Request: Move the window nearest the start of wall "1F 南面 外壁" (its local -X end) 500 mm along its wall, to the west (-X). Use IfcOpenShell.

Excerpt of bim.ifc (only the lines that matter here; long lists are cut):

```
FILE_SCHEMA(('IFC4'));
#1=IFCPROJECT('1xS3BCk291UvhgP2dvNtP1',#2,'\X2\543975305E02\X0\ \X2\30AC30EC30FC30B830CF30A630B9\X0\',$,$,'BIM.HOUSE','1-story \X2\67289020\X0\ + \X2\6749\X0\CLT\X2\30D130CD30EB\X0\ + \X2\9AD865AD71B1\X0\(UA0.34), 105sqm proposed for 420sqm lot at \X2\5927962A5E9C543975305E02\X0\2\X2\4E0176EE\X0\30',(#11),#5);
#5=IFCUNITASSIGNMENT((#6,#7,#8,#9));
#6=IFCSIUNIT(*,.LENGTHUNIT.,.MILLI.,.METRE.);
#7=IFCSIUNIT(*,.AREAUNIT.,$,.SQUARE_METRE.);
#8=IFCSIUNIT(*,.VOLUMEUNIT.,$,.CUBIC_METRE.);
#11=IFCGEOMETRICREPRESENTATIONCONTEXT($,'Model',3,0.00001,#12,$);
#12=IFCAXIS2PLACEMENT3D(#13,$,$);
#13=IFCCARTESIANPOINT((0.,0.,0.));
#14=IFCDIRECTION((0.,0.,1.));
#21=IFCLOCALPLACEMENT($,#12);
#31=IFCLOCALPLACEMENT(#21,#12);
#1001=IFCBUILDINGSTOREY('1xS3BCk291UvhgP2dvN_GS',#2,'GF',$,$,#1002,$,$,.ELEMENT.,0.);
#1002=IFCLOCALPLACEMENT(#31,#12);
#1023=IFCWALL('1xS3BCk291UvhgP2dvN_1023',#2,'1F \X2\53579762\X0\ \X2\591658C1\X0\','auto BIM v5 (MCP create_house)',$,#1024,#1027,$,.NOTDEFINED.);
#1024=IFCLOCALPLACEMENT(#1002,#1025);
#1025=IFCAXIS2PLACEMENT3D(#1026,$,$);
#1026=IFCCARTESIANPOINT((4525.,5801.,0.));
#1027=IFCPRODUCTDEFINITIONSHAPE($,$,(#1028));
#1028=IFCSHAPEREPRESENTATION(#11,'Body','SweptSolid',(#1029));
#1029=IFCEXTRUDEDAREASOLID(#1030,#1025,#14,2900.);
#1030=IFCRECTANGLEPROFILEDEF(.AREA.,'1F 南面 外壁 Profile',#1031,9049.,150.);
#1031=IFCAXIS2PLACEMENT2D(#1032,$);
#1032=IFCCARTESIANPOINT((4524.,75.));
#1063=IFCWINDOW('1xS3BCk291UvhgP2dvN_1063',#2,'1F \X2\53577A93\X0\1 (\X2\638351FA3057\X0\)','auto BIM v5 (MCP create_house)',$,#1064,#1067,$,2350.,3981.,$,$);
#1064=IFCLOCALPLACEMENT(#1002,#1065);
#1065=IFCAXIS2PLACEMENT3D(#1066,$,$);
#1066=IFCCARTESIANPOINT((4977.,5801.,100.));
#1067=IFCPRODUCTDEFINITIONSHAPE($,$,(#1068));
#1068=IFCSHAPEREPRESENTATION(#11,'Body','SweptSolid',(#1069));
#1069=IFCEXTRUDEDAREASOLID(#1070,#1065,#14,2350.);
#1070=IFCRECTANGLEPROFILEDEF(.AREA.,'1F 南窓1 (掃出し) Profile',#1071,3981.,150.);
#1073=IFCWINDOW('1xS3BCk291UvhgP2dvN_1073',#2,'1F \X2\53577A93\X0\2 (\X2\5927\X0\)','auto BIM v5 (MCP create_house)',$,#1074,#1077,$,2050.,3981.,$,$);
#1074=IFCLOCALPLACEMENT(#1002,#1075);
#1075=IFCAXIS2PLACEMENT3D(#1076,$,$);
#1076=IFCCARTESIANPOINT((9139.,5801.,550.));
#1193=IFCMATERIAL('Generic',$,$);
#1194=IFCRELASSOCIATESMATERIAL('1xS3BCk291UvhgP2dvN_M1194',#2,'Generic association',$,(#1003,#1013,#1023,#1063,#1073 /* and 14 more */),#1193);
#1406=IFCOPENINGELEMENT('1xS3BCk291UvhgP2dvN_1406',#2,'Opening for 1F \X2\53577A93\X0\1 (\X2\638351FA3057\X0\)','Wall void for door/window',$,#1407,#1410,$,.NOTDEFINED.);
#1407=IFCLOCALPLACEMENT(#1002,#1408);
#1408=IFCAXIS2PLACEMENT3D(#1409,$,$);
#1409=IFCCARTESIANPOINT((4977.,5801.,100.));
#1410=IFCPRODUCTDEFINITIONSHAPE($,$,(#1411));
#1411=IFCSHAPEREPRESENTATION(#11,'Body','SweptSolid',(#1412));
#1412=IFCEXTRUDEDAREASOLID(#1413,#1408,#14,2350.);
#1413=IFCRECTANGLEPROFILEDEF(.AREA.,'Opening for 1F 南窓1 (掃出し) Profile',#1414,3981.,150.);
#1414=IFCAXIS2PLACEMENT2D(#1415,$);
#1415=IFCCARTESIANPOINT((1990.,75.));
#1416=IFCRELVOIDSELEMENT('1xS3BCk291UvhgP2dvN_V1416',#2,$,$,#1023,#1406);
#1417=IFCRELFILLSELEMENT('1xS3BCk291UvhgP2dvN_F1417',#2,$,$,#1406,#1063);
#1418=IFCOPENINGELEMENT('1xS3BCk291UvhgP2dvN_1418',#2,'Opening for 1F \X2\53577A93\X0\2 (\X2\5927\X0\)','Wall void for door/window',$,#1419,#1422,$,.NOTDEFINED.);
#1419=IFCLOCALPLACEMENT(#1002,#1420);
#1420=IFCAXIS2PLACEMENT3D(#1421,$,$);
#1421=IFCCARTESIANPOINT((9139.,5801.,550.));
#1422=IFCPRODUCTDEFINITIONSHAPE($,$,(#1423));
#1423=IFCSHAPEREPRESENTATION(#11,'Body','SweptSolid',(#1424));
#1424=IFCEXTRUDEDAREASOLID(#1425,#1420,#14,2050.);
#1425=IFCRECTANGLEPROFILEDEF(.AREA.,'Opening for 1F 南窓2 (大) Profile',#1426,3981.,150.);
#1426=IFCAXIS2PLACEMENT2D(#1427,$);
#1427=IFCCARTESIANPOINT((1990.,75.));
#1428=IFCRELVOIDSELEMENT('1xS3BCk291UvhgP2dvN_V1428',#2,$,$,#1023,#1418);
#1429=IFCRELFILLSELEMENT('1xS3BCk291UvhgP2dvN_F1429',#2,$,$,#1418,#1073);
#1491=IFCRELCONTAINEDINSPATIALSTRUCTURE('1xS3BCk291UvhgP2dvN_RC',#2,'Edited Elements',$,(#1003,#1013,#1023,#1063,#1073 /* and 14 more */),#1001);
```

```python
import ifcopenshell
import ifcopenshell.api.geometry
import ifcopenshell.util.placement

model = ifcopenshell.open("bim.ifc")

window = model.by_guid("1xS3BCk291UvhgP2dvN_1063")
opening = window.FillsVoids[0].RelatingOpeningElement
wall = opening.VoidsElements[0].RelatingBuildingElement

wall_matrix = ifcopenshell.util.placement.get_local_placement(wall.ObjectPlacement)
shift = wall_matrix[:3, 0] * -500.0
before = ifcopenshell.util.placement.get_local_placement(window.ObjectPlacement)[:3, 3].copy()

# The window is not placed relative to its opening, so move both.
for product in (opening, window):
    matrix = ifcopenshell.util.placement.get_local_placement(product.ObjectPlacement)
    matrix[:3, 3] += shift
    ifcopenshell.api.geometry.edit_object_placement(model, product=product, matrix=matrix, is_si=False)

after = ifcopenshell.util.placement.get_local_placement(window.ObjectPlacement)[:3, 3]
print("window moved by", (after - before).round(3) + 0.0)

model.write("bim-out.ifc")
```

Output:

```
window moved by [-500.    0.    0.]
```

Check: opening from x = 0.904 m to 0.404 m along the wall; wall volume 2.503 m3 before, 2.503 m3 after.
